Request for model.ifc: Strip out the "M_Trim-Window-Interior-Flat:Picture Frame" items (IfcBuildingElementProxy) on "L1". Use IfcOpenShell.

First a look at what the model holds.

```python
import ifcopenshell
import ifcopenshell.util.element

model = ifcopenshell.open("model.ifc")
print(model.schema)
storey = next(s for s in model.by_type("IfcBuildingStorey") if s.Name == "L1")
proxies = [e for e in ifcopenshell.util.element.get_decomposition(storey) if e.is_a("IfcBuildingElementProxy")]
seen = {}
for e in proxies:
    element_type = ifcopenshell.util.element.get_type(e)
    name = element_type.Name if element_type not in (None, e) else None
    seen[name] = seen.get(name, 0) + 1
for name, count in sorted(seen.items(), key=str):
    print(count, "x", name)
```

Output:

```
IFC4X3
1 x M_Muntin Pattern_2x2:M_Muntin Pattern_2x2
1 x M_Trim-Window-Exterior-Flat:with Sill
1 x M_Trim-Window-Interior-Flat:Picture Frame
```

```python
import ifcopenshell
import ifcopenshell.api.root
import ifcopenshell.util.element

model = ifcopenshell.open("model.ifc")

storey = next(s for s in model.by_type("IfcBuildingStorey") if s.Name == "L1")
proxies = [e for e in ifcopenshell.util.element.get_decomposition(storey) if e.is_a("IfcBuildingElementProxy")]
targets = [e for e in proxies if (t := ifcopenshell.util.element.get_type(e)) not in (None, e) and t.Name == "M_Trim-Window-Interior-Flat:Picture Frame"]

for e in targets:
    ifcopenshell.api.root.remove_product(model, product=e)
print(len(targets), "removed")

model.write("model_rev.ifc")
```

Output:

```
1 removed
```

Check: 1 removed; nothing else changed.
